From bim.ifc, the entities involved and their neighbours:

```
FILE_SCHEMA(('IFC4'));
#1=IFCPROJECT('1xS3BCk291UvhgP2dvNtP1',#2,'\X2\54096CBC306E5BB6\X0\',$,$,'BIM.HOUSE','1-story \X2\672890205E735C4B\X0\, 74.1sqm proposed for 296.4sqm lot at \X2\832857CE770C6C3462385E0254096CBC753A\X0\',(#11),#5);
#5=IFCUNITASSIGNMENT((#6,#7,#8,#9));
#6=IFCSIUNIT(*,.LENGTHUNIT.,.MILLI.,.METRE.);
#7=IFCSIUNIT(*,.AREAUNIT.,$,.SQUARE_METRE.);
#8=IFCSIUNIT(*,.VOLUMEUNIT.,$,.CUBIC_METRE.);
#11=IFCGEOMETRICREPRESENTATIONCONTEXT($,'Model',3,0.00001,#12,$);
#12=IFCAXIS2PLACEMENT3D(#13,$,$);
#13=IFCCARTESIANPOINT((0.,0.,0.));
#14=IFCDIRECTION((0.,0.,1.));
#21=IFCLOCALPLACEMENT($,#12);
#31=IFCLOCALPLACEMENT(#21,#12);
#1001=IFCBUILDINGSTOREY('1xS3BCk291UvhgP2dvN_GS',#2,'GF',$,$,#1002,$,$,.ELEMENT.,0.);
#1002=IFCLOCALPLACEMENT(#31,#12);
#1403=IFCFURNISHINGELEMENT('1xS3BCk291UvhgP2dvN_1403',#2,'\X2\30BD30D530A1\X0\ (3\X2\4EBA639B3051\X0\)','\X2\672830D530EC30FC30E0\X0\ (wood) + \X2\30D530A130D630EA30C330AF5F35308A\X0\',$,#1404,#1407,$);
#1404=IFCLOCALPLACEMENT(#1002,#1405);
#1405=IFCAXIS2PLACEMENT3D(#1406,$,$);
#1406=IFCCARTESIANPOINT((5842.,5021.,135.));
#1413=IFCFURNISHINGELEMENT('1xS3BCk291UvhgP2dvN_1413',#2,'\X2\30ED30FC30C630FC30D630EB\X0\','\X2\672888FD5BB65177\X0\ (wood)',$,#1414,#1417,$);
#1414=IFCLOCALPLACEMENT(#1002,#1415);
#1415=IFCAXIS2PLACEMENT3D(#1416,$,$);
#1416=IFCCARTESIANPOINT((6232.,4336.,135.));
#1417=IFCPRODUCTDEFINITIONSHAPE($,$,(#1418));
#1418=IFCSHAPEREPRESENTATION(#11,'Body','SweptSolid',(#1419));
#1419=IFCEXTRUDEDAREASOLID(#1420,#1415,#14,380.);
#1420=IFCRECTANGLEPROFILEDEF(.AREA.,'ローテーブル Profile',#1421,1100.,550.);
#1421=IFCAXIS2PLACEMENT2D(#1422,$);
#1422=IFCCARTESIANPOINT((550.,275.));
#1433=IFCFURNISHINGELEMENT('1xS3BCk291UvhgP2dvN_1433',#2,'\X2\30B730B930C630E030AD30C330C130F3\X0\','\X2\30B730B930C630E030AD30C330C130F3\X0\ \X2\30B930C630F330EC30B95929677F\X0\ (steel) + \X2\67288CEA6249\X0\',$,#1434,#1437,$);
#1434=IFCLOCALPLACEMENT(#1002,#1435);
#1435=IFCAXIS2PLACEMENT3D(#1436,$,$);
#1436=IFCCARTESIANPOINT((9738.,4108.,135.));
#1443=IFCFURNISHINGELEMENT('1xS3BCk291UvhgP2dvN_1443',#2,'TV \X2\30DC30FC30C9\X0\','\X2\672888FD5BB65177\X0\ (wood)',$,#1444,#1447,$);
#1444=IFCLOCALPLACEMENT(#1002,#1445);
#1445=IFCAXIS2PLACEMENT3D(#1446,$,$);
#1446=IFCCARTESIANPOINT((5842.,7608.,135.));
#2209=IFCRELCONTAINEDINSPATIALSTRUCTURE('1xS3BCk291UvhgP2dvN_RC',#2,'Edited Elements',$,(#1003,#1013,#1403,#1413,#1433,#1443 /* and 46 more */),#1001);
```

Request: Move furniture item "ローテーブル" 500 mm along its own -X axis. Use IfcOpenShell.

```python
import ifcopenshell
import ifcopenshell.api.geometry
import ifcopenshell.util.placement
import ifcopenshell.util.unit

model = ifcopenshell.open("bim.ifc")
unit_scale = ifcopenshell.util.unit.calculate_unit_scale(model)

item = model.by_id(1413)
matrix = ifcopenshell.util.placement.get_local_placement(item.ObjectPlacement)
matrix[:3, 3] -= matrix[:3, 0] * 0.5 / unit_scale
ifcopenshell.api.geometry.edit_object_placement(model, product=item, matrix=matrix, is_si=False)

print(ifcopenshell.util.placement.get_local_placement(item.ObjectPlacement).round(3) + 0.0)

model.write("bim_rev.ifc")
```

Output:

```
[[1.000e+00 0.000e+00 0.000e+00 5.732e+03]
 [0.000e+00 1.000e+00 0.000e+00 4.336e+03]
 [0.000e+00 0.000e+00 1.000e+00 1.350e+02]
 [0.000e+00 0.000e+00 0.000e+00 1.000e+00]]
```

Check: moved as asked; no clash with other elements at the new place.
